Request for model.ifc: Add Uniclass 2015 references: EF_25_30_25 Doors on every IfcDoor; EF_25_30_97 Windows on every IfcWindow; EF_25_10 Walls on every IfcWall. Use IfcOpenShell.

First a look at what the model holds.

```python
import ifcopenshell

model = ifcopenshell.open("model.ifc")
print(model.schema)
print("classifications:", [c.Name for c in model.by_type("IfcClassification")])
for ifc_class in ("IfcDoor", "IfcRoof", "IfcStair", "IfcWall", "IfcWindow"):
    print(ifc_class, len(model.by_type(ifc_class)))
```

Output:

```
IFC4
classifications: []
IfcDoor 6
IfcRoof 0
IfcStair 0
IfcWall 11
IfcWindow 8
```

```python
import ifcopenshell
import ifcopenshell.api.classification

model = ifcopenshell.open("model.ifc")

system = ifcopenshell.api.classification.add_classification(model, classification="Uniclass 2015")

codes = {
    "IfcDoor": ("EF_25_30_25", "Doors"),
    "IfcWindow": ("EF_25_30_97", "Windows"),
    "IfcWall": ("EF_25_10", "Walls"),
}
for ifc_class, (code, name) in codes.items():
    products = model.by_type(ifc_class)
    ifcopenshell.api.classification.add_reference(
        model, products=products, classification=system, identification=code, name=name
    )
    print(code, len(products))

model.write("model-out.ifc")
```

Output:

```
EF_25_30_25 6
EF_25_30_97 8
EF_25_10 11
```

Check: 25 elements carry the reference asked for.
